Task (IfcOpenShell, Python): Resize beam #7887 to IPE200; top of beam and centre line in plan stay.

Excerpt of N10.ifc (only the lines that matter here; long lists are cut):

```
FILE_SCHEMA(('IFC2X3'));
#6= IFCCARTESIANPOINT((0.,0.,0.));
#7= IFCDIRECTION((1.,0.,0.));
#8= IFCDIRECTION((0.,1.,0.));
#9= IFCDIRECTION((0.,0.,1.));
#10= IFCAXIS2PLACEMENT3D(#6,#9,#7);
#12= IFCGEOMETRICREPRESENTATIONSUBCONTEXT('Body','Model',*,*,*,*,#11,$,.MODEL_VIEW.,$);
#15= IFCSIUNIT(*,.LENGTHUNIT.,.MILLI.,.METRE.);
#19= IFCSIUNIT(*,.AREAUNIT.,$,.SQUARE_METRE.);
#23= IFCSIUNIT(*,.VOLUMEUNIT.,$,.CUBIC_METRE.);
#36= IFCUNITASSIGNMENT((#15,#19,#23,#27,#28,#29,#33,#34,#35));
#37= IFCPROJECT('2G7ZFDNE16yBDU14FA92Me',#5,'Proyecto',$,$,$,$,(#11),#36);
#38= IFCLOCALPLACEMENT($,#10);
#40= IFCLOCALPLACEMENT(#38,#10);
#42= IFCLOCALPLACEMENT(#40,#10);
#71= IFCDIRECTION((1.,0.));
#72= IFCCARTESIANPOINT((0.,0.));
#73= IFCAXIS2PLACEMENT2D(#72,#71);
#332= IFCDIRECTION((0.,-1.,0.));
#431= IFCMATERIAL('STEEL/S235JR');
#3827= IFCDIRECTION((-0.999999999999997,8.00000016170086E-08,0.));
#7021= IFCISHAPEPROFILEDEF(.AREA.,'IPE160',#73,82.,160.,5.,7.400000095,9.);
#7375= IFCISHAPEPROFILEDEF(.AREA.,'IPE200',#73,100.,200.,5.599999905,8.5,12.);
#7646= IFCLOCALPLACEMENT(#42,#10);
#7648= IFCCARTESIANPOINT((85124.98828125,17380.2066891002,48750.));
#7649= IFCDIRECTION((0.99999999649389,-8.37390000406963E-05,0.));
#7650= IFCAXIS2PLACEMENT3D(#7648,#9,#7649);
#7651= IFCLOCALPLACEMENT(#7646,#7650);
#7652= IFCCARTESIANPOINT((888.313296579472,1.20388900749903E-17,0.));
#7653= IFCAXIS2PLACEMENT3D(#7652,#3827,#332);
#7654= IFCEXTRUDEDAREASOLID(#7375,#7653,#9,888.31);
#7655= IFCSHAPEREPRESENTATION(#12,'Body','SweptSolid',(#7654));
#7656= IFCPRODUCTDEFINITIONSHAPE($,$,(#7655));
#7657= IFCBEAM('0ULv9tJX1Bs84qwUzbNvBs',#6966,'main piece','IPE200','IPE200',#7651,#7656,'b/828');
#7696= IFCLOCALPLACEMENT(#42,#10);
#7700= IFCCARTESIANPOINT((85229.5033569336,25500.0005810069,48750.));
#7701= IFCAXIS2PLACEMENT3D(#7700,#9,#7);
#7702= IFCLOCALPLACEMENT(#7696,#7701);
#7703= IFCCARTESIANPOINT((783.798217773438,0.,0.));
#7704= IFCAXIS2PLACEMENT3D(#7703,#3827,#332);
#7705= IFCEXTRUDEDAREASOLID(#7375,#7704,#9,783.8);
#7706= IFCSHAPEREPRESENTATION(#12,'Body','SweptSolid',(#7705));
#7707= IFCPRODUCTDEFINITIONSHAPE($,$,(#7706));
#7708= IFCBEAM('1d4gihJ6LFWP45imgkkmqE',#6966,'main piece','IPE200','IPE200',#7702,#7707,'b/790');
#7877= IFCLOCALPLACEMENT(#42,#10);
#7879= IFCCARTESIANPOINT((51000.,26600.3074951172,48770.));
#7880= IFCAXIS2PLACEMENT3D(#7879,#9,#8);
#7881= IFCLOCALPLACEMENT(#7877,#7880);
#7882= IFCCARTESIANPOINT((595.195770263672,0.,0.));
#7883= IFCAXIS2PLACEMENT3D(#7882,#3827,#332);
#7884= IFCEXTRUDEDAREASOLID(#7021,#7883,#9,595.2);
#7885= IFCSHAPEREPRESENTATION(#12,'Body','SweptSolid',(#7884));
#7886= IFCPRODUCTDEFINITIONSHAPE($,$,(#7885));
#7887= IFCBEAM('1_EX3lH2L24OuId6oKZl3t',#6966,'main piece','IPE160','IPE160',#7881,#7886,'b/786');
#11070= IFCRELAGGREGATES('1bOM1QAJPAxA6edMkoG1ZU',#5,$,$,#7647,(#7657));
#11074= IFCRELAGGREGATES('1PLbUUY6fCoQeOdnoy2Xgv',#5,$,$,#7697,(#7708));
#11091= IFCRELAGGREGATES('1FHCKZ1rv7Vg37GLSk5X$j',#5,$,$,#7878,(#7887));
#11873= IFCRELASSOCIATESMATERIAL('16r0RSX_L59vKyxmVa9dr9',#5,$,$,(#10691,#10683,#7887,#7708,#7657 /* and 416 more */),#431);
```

```python
import ifcopenshell
import ifcopenshell.util.element
import ifcopenshell.util.representation

model = ifcopenshell.open("N10.ifc")

member = model.by_id(7887)
source = next(p for p in model.by_type("IfcIShapeProfileDef") if p.ProfileName == "IPE200")

body = ifcopenshell.util.representation.get_representation(member, "Model", "Body")
solid = body.Items[0]
old_profile = solid.SweptArea

# Copy the section's sizes but keep this member's own profile position.
profile = ifcopenshell.util.element.copy(model, source)
# Profiles are centred, so shift by half the change in depth to hold the top.
shift = (old_profile.OverallDepth - profile.OverallDepth) / 2
x, y = old_profile.Position.Location.Coordinates
up = (0.0, 1.0)  # upwards, in the solid's own plane
location = model.createIfcCartesianPoint((x + up[0] * shift, y + up[1] * shift))
profile.Position = model.createIfcAxis2Placement2D(location, old_profile.Position.RefDirection)
solid.SweptArea = profile
if not model.get_total_inverses(old_profile):
    ifcopenshell.util.element.remove_deep2(model, old_profile)
member.Description = member.Description.replace("IPE160", "IPE200")
member.ObjectType = member.ObjectType.replace("IPE160", "IPE200")

print(solid.SweptArea)

model.write("N10_updated.ifc")
```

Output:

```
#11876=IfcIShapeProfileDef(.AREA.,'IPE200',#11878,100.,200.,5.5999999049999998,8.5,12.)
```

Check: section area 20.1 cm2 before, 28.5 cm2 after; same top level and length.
